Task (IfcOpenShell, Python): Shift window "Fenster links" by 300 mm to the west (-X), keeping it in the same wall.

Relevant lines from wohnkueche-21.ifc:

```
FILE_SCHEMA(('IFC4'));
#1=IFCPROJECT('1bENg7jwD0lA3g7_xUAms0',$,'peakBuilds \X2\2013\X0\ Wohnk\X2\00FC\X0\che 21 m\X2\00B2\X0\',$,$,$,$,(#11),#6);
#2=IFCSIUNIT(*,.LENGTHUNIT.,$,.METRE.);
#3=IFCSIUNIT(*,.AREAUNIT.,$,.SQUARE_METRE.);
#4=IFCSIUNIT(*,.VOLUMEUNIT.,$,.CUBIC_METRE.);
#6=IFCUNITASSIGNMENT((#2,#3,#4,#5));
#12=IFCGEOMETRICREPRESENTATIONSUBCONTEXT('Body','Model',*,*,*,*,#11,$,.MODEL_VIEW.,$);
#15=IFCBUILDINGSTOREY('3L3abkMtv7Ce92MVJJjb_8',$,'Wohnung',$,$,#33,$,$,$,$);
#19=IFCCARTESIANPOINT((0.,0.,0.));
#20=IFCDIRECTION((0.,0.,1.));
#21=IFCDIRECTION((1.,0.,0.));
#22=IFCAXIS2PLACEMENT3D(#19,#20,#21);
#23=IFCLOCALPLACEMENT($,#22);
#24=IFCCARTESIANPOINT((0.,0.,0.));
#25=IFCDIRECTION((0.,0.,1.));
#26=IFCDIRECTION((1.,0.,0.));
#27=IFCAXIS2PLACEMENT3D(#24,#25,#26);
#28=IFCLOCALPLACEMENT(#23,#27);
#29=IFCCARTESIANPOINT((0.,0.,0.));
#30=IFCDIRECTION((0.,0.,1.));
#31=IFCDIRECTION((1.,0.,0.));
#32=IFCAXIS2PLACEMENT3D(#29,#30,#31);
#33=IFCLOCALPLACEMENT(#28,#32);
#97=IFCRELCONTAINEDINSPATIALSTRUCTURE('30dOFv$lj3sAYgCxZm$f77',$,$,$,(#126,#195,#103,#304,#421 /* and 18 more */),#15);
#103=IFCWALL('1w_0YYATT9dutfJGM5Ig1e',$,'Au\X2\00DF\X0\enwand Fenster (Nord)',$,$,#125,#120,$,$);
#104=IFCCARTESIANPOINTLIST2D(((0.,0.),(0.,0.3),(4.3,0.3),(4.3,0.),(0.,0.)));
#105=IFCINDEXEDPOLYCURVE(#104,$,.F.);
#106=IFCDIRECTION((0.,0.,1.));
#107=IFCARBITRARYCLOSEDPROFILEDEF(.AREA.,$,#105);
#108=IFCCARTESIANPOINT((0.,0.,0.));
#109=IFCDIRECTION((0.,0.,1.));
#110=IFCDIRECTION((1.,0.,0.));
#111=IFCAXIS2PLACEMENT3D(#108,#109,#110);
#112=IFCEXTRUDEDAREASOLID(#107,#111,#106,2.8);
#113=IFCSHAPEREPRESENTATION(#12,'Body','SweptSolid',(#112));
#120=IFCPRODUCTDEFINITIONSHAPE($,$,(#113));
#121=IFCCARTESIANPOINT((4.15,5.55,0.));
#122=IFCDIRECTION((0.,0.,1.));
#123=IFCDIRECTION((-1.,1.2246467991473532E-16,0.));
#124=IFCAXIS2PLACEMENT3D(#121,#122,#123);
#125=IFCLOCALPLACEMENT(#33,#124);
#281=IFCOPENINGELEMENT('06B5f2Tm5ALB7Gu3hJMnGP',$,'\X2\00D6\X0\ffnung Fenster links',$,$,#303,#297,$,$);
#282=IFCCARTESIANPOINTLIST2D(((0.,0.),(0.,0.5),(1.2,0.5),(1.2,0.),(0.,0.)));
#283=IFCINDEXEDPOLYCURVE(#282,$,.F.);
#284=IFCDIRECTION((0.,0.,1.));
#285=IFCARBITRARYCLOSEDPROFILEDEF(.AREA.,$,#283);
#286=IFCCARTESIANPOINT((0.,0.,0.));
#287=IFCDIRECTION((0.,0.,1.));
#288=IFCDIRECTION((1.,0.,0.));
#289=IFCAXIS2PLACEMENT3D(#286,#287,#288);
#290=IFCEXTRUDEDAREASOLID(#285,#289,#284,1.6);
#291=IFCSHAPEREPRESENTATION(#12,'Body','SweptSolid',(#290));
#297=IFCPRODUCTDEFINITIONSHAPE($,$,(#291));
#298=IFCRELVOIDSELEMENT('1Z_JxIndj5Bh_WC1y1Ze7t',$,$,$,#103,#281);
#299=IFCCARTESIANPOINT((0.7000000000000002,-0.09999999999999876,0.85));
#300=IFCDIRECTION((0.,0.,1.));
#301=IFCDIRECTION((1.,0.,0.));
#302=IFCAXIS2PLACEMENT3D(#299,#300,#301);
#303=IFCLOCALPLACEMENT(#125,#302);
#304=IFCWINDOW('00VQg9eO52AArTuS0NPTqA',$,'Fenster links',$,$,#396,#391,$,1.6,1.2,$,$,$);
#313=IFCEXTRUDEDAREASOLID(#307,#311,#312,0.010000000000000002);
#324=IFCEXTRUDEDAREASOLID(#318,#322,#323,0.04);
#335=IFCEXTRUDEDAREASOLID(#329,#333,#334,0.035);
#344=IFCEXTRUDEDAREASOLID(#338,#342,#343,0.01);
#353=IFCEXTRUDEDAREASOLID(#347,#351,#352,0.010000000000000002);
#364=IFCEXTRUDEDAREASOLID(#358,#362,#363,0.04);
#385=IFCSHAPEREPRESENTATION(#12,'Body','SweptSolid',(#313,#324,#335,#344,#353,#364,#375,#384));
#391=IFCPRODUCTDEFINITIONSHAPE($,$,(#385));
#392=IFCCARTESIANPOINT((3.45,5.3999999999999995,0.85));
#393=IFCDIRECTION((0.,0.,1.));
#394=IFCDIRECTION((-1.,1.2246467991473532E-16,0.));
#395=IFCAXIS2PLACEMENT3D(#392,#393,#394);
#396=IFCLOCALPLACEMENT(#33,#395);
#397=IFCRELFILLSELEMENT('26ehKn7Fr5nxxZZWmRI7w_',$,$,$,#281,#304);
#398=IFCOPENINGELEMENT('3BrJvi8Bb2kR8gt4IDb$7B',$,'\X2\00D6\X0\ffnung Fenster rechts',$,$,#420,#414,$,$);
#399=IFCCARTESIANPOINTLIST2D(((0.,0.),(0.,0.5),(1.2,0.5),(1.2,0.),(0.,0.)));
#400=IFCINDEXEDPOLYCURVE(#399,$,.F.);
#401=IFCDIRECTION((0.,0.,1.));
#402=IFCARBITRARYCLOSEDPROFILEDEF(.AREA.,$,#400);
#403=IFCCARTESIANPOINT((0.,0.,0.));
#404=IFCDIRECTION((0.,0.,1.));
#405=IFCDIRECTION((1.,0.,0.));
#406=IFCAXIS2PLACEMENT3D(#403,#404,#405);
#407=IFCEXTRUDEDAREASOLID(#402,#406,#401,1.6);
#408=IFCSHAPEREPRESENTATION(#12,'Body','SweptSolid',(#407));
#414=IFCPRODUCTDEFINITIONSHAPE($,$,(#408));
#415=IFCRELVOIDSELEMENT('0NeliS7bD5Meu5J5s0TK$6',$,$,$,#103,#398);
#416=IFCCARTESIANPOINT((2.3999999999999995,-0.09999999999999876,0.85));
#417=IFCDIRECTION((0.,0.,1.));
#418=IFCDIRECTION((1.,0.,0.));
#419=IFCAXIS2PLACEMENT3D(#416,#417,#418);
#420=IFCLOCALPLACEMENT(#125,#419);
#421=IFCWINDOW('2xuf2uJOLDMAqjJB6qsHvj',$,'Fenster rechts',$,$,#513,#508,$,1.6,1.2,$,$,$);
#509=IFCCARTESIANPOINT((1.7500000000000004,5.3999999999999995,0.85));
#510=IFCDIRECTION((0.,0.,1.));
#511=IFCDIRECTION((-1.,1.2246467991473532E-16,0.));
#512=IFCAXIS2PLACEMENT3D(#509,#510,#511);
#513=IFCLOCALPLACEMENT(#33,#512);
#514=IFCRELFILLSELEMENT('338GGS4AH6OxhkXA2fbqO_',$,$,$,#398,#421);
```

```python
import ifcopenshell
import ifcopenshell.api.geometry
import ifcopenshell.util.placement

model = ifcopenshell.open("wohnkueche-21.ifc")

window = model.by_guid("00VQg9eO52AArTuS0NPTqA")
opening = window.FillsVoids[0].RelatingOpeningElement
wall = opening.VoidsElements[0].RelatingBuildingElement

wall_matrix = ifcopenshell.util.placement.get_local_placement(wall.ObjectPlacement)
shift = wall_matrix[:3, 0] * 0.3
before = ifcopenshell.util.placement.get_local_placement(window.ObjectPlacement)[:3, 3].copy()

# The window is not placed relative to its opening, so move both.
for product in (opening, window):
    matrix = ifcopenshell.util.placement.get_local_placement(product.ObjectPlacement)
    matrix[:3, 3] += shift
    ifcopenshell.api.geometry.edit_object_placement(model, product=product, matrix=matrix, is_si=False)

after = ifcopenshell.util.placement.get_local_placement(window.ObjectPlacement)[:3, 3]
print("window moved by", (after - before).round(3) + 0.0)

model.write("wohnkueche-21_v2.ifc")
```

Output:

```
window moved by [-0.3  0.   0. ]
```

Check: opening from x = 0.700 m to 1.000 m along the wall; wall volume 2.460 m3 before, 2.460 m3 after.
